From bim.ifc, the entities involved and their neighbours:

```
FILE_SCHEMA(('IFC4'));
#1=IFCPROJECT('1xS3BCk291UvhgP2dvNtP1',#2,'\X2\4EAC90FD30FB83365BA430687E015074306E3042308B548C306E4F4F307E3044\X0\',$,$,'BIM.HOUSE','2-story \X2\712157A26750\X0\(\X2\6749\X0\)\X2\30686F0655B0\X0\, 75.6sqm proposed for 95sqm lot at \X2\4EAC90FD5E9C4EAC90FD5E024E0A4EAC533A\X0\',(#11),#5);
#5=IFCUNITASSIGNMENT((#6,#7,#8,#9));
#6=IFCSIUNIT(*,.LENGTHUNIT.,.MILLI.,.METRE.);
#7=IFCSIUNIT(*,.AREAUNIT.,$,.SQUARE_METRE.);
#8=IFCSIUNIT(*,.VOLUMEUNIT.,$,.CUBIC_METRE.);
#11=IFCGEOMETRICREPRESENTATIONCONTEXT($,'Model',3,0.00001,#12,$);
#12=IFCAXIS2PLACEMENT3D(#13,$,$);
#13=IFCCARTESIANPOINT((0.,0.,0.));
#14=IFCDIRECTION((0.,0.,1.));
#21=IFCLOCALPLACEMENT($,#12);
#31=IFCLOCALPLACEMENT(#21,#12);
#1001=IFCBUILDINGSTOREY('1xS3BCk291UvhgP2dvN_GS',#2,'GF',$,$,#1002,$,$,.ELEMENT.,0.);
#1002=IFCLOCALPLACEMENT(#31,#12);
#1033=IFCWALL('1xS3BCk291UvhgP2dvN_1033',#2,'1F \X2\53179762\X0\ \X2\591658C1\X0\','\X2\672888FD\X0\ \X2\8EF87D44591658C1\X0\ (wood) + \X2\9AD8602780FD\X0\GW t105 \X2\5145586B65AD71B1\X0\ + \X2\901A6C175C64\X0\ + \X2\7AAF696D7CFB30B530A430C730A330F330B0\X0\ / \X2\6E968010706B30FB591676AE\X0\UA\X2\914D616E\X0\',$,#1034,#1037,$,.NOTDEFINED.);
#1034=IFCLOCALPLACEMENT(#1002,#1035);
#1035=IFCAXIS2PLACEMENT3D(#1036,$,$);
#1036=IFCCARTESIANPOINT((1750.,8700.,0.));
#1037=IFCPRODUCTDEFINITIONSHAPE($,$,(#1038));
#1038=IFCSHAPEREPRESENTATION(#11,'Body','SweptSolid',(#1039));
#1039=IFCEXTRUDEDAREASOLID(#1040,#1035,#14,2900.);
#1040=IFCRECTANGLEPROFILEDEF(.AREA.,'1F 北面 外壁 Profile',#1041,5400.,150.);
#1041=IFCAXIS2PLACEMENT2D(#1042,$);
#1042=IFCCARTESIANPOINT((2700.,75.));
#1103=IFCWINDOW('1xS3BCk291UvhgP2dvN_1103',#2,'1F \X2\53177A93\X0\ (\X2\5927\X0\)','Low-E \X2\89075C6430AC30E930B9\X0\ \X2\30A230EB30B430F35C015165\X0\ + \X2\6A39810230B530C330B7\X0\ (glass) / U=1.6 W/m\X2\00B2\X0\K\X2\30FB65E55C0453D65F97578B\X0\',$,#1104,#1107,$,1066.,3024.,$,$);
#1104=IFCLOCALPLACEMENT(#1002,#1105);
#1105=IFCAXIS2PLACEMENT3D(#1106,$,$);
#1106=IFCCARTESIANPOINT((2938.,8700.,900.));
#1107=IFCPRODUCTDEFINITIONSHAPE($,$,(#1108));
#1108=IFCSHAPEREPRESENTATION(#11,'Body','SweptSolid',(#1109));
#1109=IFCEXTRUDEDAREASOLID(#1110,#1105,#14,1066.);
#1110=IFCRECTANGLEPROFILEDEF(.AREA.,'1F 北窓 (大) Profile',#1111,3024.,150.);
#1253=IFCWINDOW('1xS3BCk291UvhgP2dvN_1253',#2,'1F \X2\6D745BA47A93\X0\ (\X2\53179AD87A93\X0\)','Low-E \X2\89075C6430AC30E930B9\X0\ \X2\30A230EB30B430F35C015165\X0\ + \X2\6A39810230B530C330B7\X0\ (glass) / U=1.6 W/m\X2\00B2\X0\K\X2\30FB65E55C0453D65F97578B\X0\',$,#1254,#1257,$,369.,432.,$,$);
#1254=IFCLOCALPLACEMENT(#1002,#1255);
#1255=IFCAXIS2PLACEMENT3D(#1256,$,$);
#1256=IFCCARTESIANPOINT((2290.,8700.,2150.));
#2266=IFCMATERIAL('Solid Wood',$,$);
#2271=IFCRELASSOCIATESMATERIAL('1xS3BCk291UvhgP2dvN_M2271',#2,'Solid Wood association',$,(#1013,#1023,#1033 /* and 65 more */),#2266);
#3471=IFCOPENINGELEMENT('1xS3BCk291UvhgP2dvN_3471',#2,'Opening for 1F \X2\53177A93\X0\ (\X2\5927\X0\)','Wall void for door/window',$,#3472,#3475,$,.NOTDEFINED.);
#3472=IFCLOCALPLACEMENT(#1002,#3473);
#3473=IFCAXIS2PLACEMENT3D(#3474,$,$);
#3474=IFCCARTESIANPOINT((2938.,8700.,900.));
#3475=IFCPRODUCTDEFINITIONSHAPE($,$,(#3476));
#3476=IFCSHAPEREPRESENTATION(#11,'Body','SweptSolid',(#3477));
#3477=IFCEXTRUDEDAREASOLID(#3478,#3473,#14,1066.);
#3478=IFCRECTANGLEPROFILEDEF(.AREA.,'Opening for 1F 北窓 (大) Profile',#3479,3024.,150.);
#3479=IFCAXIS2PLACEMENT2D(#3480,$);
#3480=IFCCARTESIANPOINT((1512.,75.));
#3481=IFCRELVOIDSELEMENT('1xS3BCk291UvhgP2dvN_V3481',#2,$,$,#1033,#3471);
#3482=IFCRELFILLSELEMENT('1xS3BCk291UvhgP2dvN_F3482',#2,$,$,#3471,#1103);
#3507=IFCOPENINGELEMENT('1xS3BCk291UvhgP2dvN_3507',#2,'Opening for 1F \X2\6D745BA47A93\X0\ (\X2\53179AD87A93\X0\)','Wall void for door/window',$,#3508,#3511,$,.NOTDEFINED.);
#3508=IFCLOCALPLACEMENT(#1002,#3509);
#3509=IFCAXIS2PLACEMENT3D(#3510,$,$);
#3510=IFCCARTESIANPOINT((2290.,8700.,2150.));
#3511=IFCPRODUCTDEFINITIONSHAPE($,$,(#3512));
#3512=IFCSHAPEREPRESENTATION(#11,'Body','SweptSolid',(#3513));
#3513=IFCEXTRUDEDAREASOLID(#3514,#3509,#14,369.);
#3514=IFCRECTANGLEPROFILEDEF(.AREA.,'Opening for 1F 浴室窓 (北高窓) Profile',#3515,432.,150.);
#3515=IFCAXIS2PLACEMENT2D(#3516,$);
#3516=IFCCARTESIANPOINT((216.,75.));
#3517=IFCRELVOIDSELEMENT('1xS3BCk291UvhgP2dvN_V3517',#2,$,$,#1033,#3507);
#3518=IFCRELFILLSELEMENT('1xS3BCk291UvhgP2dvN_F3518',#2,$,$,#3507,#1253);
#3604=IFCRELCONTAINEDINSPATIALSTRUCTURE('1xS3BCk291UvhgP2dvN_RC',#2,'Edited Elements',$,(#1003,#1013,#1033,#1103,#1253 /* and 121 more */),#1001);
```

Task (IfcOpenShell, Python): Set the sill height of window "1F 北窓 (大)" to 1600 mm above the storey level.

```python
import numpy as np
import ifcopenshell
import ifcopenshell.api.geometry
import ifcopenshell.geom
import ifcopenshell.util.element
import ifcopenshell.util.placement
import ifcopenshell.util.shape
import ifcopenshell.util.unit

model = ifcopenshell.open("bim.ifc")
unit_scale = ifcopenshell.util.unit.calculate_unit_scale(model)

window = model.by_guid("1xS3BCk291UvhgP2dvN_1103")
opening = window.FillsVoids[0].RelatingOpeningElement
storey = ifcopenshell.util.element.get_container(window, ifc_class="IfcBuildingStorey")
level = ifcopenshell.util.placement.get_local_placement(storey.ObjectPlacement)[2, 3]

# The opening's origin need not be at the sill, so measure its lowest point.
shape = ifcopenshell.geom.create_shape(ifcopenshell.geom.settings(), opening)
bottom = ifcopenshell.util.shape.get_shape_bottom_elevation(shape, shape.geometry) / unit_scale
dz = level + 1.6 / unit_scale - bottom

shift = np.array([0.0, 0.0, dz])
# The window is not placed relative to its opening, so move both.
for product in (opening, window):
    matrix = ifcopenshell.util.placement.get_local_placement(product.ObjectPlacement)
    matrix[:3, 3] += shift
    ifcopenshell.api.geometry.edit_object_placement(model, product=product, matrix=matrix, is_si=False)

print(f"moved by {dz * unit_scale:+.3f} m")

model.write("bim_rev.ifc")
```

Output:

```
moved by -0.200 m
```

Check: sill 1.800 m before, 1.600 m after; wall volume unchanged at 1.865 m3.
